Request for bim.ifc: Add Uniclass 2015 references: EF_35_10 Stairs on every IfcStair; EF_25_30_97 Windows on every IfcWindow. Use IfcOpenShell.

First a look at what the model holds.

```python
import ifcopenshell

model = ifcopenshell.open("bim.ifc")
print(model.schema)
print("classifications:", [c.Name for c in model.by_type("IfcClassification")])
for ifc_class in ("IfcDoor", "IfcRoof", "IfcStair", "IfcWall", "IfcWindow"):
    print(ifc_class, len(model.by_type(ifc_class)))
```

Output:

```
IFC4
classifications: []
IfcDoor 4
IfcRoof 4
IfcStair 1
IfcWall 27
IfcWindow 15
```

```python
import ifcopenshell
import ifcopenshell.api.classification

model = ifcopenshell.open("bim.ifc")

system = ifcopenshell.api.classification.add_classification(model, classification="Uniclass 2015")

codes = {
    "IfcStair": ("EF_35_10", "Stairs"),
    "IfcWindow": ("EF_25_30_97", "Windows"),
}
for ifc_class, (code, name) in codes.items():
    products = model.by_type(ifc_class)
    ifcopenshell.api.classification.add_reference(
        model, products=products, classification=system, identification=code, name=name
    )
    print(code, len(products))

model.write("bim_rev.ifc")
```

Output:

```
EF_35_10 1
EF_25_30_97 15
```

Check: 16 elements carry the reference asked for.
